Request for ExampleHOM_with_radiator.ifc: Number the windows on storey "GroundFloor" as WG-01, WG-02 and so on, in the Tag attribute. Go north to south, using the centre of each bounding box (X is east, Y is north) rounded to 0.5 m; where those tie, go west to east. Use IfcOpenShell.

First a look at what the model holds.

```python
import ifcopenshell
import ifcopenshell.util.element
import ifcopenshell.util.placement

model = ifcopenshell.open("ExampleHOM_with_radiator.ifc")
print(model.schema)
storey = next(s for s in model.by_type("IfcBuildingStorey") if s.Name == "GroundFloor")
windows = [e for e in ifcopenshell.util.element.get_decomposition(storey) if e.is_a("IfcWindow")]
for e in sorted(windows, key=lambda e: e.id()):
    origin = ifcopenshell.util.placement.get_local_placement(e.ObjectPlacement)[:3, 3]
    print(e.id(), e.Tag, e.Name, origin.round(2) + 0.0, sep=" | ")
```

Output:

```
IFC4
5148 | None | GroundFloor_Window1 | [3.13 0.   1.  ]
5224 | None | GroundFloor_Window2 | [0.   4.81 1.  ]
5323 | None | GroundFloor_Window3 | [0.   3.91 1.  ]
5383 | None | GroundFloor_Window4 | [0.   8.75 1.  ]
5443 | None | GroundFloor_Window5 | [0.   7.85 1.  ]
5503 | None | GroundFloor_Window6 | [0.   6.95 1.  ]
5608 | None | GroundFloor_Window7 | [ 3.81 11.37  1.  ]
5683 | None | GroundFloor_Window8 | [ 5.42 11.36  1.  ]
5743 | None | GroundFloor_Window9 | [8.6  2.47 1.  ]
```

```python
import ifcopenshell
import ifcopenshell.geom
import ifcopenshell.util.element
import ifcopenshell.util.shape

model = ifcopenshell.open("ExampleHOM_with_radiator.ifc")
settings = ifcopenshell.geom.settings()
settings.set("use-world-coords", True)


def centre(element):
    shape = ifcopenshell.geom.create_shape(settings, element)
    return ifcopenshell.util.shape.get_bbox_centroid(shape.geometry)


storey = next(s for s in model.by_type("IfcBuildingStorey") if s.Name == "GroundFloor")
windows = [e for e in ifcopenshell.util.element.get_decomposition(storey) if e.is_a("IfcWindow")]

# Insertion points can sit at a corner or the storey origin, so sort by the geometry (in metres).
centres = {e: centre(e) for e in windows}
windows.sort(key=lambda e: (-round(centres[e][1] / 0.5), centres[e][0]))

for i, e in enumerate(windows, start=1):
    number = f"WG-{i:02d}"
    e.Tag = number
    print(e.id(), number)

model.write("ExampleHOM_with_radiator-out.ifc")
```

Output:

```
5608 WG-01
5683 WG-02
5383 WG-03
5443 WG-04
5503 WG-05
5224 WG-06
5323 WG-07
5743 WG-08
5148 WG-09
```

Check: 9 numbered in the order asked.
